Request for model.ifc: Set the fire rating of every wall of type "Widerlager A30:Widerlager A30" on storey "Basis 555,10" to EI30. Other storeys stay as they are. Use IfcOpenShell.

First a look at what the model holds.

```python
import ifcopenshell
import ifcopenshell.util.element

model = ifcopenshell.open("model.ifc")
print(model.schema)
storey = next(s for s in model.by_type("IfcBuildingStorey") if s.Name == "Basis 555,10")
walls = [e for e in ifcopenshell.util.element.get_decomposition(storey) if e.is_a("IfcWall")]
seen = {}
for e in walls:
    element_type = ifcopenshell.util.element.get_type(e)
    key = (element_type.Name if element_type != e and element_type else None, ifcopenshell.util.element.get_pset(e, "Pset_WallCommon", "FireRating"))
    seen[key] = seen.get(key, 0) + 1
for (name, value), count in sorted(seen.items(), key=str):
    print(count, "x", name, "|", value)
```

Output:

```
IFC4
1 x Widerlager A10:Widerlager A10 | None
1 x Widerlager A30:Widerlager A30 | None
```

```python
import ifcopenshell
import ifcopenshell.api.pset
import ifcopenshell.util.element

model = ifcopenshell.open("model.ifc")

storey = next(s for s in model.by_type("IfcBuildingStorey") if s.Name == "Basis 555,10")
walls = [e for e in ifcopenshell.util.element.get_decomposition(storey) if e.is_a("IfcWall")]

count = 0
for e in walls:
    element_type = ifcopenshell.util.element.get_type(e)
    if element_type in (None, e) or element_type.Name != "Widerlager A30:Widerlager A30":
        continue
    # add_pset returns the element's existing set when there is one.
    pset = ifcopenshell.api.pset.add_pset(model, product=e, name="Pset_WallCommon")
    ifcopenshell.api.pset.edit_pset(model, pset=pset, properties={"FireRating": "EI30"})
    count += 1

print(count, "walls updated")

model.write("model_v2.ifc")
```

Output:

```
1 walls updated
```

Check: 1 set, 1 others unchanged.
